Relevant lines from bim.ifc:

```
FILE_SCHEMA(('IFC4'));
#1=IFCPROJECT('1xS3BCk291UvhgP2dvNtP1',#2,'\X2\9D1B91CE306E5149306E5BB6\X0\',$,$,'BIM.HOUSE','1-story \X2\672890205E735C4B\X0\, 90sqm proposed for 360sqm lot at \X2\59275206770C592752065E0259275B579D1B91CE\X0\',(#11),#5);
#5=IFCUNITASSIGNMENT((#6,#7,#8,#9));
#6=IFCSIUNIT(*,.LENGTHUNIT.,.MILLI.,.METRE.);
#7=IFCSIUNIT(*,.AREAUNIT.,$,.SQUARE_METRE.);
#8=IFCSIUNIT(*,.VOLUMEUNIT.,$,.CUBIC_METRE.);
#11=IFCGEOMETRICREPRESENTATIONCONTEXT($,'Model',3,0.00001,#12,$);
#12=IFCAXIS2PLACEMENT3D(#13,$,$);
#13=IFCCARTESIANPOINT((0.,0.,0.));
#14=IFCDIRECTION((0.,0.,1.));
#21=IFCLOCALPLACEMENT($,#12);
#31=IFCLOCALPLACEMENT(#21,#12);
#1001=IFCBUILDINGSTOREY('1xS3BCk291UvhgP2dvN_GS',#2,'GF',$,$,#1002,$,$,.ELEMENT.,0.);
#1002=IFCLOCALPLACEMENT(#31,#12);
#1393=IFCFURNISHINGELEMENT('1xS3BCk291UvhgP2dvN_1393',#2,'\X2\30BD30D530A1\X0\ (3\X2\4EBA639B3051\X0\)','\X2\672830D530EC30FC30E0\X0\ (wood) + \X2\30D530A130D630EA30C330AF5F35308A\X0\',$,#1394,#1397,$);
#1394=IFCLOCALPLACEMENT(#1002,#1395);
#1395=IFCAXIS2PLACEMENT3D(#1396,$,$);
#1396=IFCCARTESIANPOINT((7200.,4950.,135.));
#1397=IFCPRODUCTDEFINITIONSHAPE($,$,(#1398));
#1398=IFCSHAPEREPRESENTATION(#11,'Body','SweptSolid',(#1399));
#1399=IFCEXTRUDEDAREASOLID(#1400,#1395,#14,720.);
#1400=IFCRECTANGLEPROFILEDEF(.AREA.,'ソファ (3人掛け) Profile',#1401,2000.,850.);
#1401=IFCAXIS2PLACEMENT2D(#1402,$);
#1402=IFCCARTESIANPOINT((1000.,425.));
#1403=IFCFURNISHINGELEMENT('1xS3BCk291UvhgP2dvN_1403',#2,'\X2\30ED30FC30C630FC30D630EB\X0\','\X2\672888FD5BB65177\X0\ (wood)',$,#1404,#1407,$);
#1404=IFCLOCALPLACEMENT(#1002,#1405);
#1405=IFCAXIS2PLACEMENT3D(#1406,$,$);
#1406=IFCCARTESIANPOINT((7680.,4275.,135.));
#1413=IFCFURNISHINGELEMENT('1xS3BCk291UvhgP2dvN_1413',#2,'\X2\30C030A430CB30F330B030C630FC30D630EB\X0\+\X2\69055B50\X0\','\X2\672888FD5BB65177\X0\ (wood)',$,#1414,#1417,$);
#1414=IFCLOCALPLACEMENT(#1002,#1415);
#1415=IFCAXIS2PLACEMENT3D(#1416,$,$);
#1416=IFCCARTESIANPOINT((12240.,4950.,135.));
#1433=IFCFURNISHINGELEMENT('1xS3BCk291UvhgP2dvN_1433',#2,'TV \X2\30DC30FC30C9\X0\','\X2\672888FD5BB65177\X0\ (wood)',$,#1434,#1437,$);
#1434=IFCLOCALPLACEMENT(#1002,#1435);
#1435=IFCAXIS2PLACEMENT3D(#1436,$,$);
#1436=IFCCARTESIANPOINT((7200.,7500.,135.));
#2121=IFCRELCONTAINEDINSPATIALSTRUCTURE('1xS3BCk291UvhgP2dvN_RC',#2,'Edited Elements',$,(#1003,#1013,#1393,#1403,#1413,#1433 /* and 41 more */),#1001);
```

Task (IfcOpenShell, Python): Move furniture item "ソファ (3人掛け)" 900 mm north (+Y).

```python
import ifcopenshell
import ifcopenshell.api.geometry
import ifcopenshell.util.placement
import ifcopenshell.util.unit

model = ifcopenshell.open("bim.ifc")
unit_scale = ifcopenshell.util.unit.calculate_unit_scale(model)

item = model.by_guid("1xS3BCk291UvhgP2dvN_1393")
matrix = ifcopenshell.util.placement.get_local_placement(item.ObjectPlacement)
matrix[1, 3] += 0.9 / unit_scale
ifcopenshell.api.geometry.edit_object_placement(model, product=item, matrix=matrix, is_si=False)

print(ifcopenshell.util.placement.get_local_placement(item.ObjectPlacement).round(3) + 0.0)

model.write("bim_updated.ifc")
```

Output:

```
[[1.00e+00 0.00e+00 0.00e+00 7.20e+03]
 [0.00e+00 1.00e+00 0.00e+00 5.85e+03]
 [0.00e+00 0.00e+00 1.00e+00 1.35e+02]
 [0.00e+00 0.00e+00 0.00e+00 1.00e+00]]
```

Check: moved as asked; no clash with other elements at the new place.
